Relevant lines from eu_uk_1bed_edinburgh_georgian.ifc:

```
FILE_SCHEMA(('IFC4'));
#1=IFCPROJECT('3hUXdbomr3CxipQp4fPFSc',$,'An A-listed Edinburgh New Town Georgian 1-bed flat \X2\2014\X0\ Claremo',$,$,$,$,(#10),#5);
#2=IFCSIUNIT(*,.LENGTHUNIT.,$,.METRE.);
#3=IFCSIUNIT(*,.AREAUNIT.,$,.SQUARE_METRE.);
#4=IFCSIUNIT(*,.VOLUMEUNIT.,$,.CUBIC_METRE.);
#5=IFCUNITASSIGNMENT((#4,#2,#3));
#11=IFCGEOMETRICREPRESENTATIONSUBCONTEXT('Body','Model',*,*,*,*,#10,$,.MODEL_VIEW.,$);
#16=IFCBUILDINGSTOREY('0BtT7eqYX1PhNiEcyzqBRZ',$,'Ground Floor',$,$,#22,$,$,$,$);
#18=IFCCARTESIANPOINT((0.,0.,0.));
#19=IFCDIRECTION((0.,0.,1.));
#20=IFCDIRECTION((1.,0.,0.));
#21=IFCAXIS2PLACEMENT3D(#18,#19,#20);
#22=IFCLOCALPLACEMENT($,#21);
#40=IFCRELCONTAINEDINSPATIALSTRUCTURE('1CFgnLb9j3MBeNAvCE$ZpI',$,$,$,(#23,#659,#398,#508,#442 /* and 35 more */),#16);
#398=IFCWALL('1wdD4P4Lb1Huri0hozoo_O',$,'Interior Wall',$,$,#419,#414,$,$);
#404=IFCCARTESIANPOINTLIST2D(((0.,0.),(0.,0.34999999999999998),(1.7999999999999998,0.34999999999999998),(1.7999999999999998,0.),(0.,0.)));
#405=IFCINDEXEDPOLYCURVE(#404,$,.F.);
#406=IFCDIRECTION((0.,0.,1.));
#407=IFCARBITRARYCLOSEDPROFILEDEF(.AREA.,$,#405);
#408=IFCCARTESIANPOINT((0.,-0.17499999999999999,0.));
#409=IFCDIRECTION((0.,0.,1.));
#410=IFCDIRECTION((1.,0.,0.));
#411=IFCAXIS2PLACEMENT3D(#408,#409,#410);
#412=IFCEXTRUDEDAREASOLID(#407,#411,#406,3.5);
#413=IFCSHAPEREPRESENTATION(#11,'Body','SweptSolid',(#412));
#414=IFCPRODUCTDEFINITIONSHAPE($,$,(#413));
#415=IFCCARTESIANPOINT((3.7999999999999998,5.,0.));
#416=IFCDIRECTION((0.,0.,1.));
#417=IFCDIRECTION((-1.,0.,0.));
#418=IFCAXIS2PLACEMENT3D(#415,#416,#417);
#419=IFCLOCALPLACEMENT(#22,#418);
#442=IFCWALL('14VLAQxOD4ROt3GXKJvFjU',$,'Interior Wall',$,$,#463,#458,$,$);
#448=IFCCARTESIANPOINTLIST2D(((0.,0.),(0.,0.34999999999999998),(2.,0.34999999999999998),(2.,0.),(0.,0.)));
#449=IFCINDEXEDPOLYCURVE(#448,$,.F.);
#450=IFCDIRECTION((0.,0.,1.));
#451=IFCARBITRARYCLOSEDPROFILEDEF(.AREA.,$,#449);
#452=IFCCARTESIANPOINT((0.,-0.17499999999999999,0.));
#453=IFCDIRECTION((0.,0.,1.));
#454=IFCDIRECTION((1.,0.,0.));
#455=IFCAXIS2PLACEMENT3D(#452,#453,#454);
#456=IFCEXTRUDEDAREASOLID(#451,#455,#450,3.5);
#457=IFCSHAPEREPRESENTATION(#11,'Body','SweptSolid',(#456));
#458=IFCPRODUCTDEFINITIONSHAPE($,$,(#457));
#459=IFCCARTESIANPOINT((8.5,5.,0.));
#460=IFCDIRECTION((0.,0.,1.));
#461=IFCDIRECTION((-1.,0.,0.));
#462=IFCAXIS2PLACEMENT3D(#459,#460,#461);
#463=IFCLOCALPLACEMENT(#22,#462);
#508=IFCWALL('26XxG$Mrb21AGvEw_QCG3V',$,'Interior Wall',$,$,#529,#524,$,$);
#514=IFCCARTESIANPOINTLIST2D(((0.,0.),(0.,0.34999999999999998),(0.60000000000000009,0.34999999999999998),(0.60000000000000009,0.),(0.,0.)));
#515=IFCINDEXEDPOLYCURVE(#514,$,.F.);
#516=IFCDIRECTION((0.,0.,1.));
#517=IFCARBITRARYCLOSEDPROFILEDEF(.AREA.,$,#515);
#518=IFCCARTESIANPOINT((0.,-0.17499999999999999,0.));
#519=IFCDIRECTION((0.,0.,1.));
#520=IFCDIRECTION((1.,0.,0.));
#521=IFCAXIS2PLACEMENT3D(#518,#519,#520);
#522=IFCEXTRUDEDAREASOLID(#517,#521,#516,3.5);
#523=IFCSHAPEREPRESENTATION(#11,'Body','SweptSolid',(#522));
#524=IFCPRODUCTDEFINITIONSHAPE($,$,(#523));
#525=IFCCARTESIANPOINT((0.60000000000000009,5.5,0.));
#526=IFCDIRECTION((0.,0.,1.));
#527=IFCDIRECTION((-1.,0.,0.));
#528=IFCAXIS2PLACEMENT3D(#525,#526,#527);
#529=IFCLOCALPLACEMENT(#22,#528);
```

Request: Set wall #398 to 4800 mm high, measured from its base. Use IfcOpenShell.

```python
import ifcopenshell
import ifcopenshell.geom
import ifcopenshell.util.representation
import ifcopenshell.util.shape
import ifcopenshell.util.unit

model = ifcopenshell.open("eu_uk_1bed_edinburgh_georgian.ifc")
unit_scale = ifcopenshell.util.unit.calculate_unit_scale(model)
settings = ifcopenshell.geom.settings()


def volume(element):
    """Net volume in cubic metres, openings subtracted."""
    shape = ifcopenshell.geom.create_shape(settings, element)
    return ifcopenshell.util.shape.get_volume(shape.geometry)


wall = model.by_guid("1wdD4P4Lb1Huri0hozoo_O")
before = volume(wall)

body = ifcopenshell.util.representation.get_representation(wall, "Model", "Body")
solid = body.Items[0]
old_height = solid.Depth
solid.Depth = 4.8 / unit_scale
after = volume(wall)

print(f"height {old_height:g} -> {solid.Depth:g}, volume {before:.3f} -> {after:.3f} m3")

model.write("eu_uk_1bed_edinburgh_georgian_edited.ifc")
```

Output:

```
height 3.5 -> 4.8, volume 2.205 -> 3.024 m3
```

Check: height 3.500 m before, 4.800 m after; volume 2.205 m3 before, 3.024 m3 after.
